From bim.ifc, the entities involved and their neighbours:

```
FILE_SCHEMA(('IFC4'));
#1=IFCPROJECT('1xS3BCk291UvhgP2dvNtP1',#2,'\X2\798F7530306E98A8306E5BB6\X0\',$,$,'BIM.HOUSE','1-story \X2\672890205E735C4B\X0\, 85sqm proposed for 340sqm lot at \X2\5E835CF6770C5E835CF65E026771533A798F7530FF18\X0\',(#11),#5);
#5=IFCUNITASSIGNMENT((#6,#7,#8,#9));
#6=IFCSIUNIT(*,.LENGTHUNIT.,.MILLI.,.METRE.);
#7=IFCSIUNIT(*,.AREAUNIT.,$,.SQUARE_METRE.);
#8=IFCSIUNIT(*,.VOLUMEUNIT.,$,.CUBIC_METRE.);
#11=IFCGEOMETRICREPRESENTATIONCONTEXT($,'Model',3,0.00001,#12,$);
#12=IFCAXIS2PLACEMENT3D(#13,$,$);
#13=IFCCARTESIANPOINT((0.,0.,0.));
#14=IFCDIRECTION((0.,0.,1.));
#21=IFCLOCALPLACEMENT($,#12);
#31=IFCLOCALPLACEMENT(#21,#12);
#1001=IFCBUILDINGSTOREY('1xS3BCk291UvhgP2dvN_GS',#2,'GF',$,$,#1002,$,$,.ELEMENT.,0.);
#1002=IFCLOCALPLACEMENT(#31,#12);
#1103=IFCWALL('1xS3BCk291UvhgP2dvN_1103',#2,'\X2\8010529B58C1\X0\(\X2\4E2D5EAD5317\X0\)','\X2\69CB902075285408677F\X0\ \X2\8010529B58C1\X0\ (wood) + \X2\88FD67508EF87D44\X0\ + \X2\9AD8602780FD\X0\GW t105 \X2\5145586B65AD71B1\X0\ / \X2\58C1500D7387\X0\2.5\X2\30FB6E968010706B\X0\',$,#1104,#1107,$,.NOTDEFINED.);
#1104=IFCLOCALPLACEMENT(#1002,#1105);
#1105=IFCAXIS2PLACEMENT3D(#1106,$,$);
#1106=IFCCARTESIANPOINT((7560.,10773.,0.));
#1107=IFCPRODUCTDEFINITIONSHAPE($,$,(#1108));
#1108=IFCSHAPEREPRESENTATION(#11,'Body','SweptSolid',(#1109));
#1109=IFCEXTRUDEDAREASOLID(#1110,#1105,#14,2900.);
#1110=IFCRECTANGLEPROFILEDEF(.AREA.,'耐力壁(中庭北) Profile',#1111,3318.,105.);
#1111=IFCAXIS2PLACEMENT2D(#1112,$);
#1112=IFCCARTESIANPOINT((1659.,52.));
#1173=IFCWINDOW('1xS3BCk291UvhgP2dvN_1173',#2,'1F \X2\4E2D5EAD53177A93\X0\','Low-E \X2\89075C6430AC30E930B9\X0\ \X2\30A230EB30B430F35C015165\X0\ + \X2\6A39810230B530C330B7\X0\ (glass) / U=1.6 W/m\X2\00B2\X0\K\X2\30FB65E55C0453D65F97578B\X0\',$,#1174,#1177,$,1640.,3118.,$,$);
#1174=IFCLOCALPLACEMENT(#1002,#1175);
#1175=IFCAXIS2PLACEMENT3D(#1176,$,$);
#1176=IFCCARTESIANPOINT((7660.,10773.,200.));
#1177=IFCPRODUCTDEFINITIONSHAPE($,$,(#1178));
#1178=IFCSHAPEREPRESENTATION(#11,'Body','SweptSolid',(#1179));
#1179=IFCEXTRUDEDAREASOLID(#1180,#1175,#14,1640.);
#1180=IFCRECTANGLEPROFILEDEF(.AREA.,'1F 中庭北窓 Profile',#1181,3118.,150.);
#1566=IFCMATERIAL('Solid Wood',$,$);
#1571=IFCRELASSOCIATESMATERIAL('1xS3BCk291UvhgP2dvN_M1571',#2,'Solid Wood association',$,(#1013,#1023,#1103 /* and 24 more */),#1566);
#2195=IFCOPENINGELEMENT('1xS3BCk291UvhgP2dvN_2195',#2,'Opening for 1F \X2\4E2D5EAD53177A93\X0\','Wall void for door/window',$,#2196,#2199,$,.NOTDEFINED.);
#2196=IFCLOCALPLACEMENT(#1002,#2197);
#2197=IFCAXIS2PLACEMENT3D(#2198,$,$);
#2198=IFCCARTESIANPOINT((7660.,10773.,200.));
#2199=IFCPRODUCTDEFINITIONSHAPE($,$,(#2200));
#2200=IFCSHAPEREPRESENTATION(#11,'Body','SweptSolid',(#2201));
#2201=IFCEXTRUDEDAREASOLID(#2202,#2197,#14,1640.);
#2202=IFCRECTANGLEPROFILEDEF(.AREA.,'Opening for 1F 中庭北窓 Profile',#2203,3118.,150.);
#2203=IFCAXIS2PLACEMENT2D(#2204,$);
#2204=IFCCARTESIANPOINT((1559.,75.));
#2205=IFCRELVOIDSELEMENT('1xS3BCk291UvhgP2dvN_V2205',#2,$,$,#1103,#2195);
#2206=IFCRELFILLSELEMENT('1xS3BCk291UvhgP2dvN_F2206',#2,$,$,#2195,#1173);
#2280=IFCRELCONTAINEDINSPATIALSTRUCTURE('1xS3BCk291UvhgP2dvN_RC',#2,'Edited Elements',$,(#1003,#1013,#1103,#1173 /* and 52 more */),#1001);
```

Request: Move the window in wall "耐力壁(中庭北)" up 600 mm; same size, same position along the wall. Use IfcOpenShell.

```python
import numpy as np
import ifcopenshell
import ifcopenshell.api.geometry
import ifcopenshell.util.placement
import ifcopenshell.util.unit

model = ifcopenshell.open("bim.ifc")
unit_scale = ifcopenshell.util.unit.calculate_unit_scale(model)

window = model.by_guid("1xS3BCk291UvhgP2dvN_1173")
opening = window.FillsVoids[0].RelatingOpeningElement
dz = 600.0

shift = np.array([0.0, 0.0, dz])
# The window is not placed relative to its opening, so move both.
for product in (opening, window):
    matrix = ifcopenshell.util.placement.get_local_placement(product.ObjectPlacement)
    matrix[:3, 3] += shift
    ifcopenshell.api.geometry.edit_object_placement(model, product=product, matrix=matrix, is_si=False)

print(f"moved by {dz * unit_scale:+.3f} m")

model.write("bim_edited.ifc")
```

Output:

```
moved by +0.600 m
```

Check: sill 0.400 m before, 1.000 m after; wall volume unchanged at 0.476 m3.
